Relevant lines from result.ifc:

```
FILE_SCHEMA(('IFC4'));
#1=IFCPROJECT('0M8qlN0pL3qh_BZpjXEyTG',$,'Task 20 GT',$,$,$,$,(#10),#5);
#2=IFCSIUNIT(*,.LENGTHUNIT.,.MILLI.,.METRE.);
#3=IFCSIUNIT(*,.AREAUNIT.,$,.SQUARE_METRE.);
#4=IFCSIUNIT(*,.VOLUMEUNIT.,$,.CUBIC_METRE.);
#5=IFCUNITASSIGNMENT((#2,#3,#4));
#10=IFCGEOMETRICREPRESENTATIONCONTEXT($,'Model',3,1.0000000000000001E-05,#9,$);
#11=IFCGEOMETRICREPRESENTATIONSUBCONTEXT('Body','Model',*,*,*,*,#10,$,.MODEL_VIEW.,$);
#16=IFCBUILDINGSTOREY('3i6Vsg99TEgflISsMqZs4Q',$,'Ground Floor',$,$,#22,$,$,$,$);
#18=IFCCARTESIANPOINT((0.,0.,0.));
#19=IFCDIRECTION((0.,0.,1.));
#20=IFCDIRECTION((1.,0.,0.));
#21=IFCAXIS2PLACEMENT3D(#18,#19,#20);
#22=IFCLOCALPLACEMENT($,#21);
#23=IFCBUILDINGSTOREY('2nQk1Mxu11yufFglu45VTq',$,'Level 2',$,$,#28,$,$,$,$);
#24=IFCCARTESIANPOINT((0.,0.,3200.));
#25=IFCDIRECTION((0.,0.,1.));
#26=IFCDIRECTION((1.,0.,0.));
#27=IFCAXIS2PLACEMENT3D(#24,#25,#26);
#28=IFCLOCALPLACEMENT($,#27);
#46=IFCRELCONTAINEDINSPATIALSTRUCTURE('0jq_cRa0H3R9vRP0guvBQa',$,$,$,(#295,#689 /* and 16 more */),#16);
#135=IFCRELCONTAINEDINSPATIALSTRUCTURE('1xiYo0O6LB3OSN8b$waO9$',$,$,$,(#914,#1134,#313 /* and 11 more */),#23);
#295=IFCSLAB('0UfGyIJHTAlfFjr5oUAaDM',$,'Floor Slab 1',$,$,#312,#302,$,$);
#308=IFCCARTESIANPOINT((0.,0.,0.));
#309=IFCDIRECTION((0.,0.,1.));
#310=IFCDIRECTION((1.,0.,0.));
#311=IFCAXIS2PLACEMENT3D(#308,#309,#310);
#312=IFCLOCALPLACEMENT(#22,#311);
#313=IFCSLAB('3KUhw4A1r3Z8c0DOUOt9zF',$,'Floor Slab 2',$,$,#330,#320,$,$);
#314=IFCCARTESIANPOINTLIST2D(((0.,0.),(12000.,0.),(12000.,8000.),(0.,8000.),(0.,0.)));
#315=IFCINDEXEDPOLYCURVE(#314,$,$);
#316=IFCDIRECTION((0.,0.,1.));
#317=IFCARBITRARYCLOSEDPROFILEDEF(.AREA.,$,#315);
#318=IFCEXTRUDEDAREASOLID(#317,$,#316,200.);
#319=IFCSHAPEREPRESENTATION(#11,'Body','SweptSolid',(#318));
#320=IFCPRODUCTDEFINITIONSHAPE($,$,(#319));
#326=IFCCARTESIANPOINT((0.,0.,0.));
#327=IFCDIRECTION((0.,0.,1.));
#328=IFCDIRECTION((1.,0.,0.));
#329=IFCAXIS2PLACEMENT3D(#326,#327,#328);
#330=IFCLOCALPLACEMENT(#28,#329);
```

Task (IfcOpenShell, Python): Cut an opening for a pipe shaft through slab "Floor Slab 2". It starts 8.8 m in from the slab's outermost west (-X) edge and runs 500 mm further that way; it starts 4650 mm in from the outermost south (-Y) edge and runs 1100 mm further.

```python
import numpy as np
import ifcopenshell
import ifcopenshell.api.feature
import ifcopenshell.api.geometry
import ifcopenshell.api.root
import ifcopenshell.geom
import ifcopenshell.util.placement
import ifcopenshell.util.representation
import ifcopenshell.util.shape
import ifcopenshell.util.unit

model = ifcopenshell.open("result.ifc")
unit_scale = ifcopenshell.util.unit.calculate_unit_scale(model)
settings = ifcopenshell.geom.settings()


def volume(element):
    """Net volume in cubic metres, openings subtracted."""
    shape = ifcopenshell.geom.create_shape(settings, element)
    return ifcopenshell.util.shape.get_volume(shape.geometry)


slab = model.by_id(313)
before = volume(slab)

# Extent in the slab's own axes, in metres. The edges named are its -X and -Y sides.
slab_shape = ifcopenshell.geom.create_shape(settings, slab)
vertices = ifcopenshell.util.shape.get_vertices(slab_shape.geometry)
x_min, y_min, bottom = vertices.min(axis=0)
top = vertices[:, 2].max()

opening = ifcopenshell.api.root.create_entity(model, ifc_class="IfcOpeningElement", name="Pipe shaft opening", predefined_type="OPENING")
context = ifcopenshell.util.representation.get_context(model, "Model", "Body", "MODEL_VIEW")
width, depth = 0.5, 1.1
outline = [(0.0, 0.0), (width, 0.0), (width, depth), (0.0, depth), (0.0, 0.0)]
# Overshoot both faces by 50 mm so the cut is clean.
shape = ifcopenshell.api.geometry.add_slab_representation(
    model, context=context, depth=top - bottom + 0.1, polyline=outline
)
ifcopenshell.api.geometry.assign_representation(model, product=opening, representation=shape)

matrix = ifcopenshell.util.placement.get_local_placement(slab.ObjectPlacement)
matrix[:, 3] = matrix @ np.append(np.array([x_min + 8.8, y_min + 4.65, bottom - 0.05]) / unit_scale, 1.0)
ifcopenshell.api.geometry.edit_object_placement(model, product=opening, matrix=matrix, is_si=False)
ifcopenshell.api.feature.add_feature(model, feature=opening, element=slab)

after = volume(slab)

print(f"slab volume {before:.3f} -> {after:.3f} m3")

model.write("result-out.ifc")
```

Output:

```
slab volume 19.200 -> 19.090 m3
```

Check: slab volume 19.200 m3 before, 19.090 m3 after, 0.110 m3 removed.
